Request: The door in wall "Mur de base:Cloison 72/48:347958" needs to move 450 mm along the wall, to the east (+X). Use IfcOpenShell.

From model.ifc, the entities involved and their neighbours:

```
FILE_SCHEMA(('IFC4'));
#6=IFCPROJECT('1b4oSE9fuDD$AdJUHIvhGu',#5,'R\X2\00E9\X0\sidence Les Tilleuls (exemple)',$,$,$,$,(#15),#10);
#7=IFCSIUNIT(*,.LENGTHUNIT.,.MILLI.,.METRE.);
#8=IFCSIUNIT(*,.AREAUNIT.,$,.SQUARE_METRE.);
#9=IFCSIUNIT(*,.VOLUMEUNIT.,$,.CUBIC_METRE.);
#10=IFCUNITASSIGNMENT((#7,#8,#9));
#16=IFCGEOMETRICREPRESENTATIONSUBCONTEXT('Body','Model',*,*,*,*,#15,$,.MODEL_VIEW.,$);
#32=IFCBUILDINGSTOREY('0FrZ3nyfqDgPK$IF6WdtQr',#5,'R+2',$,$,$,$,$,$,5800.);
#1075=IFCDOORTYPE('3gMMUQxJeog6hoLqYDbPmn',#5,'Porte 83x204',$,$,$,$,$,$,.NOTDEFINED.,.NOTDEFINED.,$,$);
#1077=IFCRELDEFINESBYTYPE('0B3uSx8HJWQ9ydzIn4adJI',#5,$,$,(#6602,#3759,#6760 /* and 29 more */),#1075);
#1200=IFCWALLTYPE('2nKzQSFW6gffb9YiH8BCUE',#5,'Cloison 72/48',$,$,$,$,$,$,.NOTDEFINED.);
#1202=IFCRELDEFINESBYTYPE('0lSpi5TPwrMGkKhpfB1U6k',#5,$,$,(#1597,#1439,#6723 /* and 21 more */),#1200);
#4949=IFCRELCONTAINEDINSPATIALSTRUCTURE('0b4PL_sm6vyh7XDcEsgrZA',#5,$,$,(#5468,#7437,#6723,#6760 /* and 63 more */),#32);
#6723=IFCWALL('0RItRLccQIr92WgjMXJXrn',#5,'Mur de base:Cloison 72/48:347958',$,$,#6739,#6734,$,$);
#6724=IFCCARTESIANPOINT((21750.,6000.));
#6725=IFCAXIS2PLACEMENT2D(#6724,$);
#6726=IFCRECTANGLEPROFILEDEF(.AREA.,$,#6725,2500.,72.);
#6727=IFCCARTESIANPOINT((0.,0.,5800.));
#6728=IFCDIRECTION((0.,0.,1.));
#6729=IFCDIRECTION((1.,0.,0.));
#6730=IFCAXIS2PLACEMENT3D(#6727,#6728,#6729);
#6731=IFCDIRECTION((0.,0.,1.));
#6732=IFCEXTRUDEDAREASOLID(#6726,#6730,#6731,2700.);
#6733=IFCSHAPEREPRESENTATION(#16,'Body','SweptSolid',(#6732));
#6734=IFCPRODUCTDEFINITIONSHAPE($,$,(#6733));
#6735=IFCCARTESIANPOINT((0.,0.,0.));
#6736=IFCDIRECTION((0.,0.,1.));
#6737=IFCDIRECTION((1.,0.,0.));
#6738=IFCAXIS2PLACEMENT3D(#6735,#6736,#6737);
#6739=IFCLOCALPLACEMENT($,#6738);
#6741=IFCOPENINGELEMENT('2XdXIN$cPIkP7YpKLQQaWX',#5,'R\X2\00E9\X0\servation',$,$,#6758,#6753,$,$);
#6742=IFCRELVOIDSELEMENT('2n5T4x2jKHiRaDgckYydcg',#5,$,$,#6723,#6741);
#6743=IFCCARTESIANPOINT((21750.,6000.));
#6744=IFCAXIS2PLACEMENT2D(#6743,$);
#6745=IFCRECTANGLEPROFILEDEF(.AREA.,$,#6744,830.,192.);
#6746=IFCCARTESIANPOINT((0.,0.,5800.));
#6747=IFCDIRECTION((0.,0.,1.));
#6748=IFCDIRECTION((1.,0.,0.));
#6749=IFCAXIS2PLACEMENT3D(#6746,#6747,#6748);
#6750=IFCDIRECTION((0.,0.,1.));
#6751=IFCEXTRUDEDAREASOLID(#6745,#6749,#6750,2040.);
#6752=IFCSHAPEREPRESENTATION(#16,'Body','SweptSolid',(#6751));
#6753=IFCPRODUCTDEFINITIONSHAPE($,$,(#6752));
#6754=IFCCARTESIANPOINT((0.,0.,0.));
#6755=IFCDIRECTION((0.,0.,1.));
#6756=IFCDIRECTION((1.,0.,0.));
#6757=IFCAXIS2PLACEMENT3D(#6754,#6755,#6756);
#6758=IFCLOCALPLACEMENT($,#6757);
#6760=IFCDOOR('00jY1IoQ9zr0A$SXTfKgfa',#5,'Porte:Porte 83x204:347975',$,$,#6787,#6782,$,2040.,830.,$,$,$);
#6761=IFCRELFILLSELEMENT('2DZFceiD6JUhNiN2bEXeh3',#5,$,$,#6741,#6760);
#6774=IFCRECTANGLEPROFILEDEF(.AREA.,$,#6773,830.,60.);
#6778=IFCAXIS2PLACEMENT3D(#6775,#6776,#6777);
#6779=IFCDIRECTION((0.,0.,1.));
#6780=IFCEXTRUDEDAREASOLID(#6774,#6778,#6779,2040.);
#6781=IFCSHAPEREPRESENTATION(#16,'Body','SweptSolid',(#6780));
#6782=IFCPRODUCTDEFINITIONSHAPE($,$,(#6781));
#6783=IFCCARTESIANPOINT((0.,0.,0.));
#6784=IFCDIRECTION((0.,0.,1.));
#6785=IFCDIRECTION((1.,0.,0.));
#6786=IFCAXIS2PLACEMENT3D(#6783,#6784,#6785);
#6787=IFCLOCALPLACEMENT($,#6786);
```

```python
import ifcopenshell
import ifcopenshell.api.geometry
import ifcopenshell.util.placement
import ifcopenshell.util.unit

model = ifcopenshell.open("model.ifc")
unit_scale = ifcopenshell.util.unit.calculate_unit_scale(model)

door = model.by_guid("00jY1IoQ9zr0A$SXTfKgfa")
opening = door.FillsVoids[0].RelatingOpeningElement
wall = opening.VoidsElements[0].RelatingBuildingElement

wall_matrix = ifcopenshell.util.placement.get_local_placement(wall.ObjectPlacement)
shift = wall_matrix[:3, 0] * 0.45 / unit_scale
before = ifcopenshell.util.placement.get_local_placement(door.ObjectPlacement)[:3, 3].copy()

# The door is not placed relative to its opening, so move both.
for product in (opening, door):
    matrix = ifcopenshell.util.placement.get_local_placement(product.ObjectPlacement)
    matrix[:3, 3] += shift
    ifcopenshell.api.geometry.edit_object_placement(model, product=product, matrix=matrix, is_si=False)

after = ifcopenshell.util.placement.get_local_placement(door.ObjectPlacement)[:3, 3]
print("door moved by", (after - before).round(3) + 0.0)

model.write("model_rev.ifc")
```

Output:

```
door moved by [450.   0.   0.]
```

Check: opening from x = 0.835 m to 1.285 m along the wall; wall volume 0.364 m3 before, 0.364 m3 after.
